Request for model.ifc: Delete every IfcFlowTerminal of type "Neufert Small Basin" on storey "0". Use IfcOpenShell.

First a look at what the model holds.

```python
import ifcopenshell
import ifcopenshell.util.element

model = ifcopenshell.open("model.ifc")
print(model.schema)
storey = next(s for s in model.by_type("IfcBuildingStorey") if s.Name == "0")
terminals = [e for e in ifcopenshell.util.element.get_decomposition(storey) if e.is_a("IfcFlowTerminal")]
seen = {}
for e in terminals:
    element_type = ifcopenshell.util.element.get_type(e)
    name = element_type.Name if element_type not in (None, e) else None
    seen[name] = seen.get(name, 0) + 1
for name, count in sorted(seen.items(), key=str):
    print(count, "x", name)
```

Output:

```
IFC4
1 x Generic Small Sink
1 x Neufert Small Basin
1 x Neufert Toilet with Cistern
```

```python
import ifcopenshell
import ifcopenshell.api.root
import ifcopenshell.util.element

model = ifcopenshell.open("model.ifc")

storey = next(s for s in model.by_type("IfcBuildingStorey") if s.Name == "0")
terminals = [e for e in ifcopenshell.util.element.get_decomposition(storey) if e.is_a("IfcFlowTerminal")]
targets = [e for e in terminals if (t := ifcopenshell.util.element.get_type(e)) not in (None, e) and t.Name == "Neufert Small Basin"]

for e in targets:
    ifcopenshell.api.root.remove_product(model, product=e)
print(len(targets), "removed")

model.write("model_edited.ifc")
```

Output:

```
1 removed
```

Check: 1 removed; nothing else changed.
